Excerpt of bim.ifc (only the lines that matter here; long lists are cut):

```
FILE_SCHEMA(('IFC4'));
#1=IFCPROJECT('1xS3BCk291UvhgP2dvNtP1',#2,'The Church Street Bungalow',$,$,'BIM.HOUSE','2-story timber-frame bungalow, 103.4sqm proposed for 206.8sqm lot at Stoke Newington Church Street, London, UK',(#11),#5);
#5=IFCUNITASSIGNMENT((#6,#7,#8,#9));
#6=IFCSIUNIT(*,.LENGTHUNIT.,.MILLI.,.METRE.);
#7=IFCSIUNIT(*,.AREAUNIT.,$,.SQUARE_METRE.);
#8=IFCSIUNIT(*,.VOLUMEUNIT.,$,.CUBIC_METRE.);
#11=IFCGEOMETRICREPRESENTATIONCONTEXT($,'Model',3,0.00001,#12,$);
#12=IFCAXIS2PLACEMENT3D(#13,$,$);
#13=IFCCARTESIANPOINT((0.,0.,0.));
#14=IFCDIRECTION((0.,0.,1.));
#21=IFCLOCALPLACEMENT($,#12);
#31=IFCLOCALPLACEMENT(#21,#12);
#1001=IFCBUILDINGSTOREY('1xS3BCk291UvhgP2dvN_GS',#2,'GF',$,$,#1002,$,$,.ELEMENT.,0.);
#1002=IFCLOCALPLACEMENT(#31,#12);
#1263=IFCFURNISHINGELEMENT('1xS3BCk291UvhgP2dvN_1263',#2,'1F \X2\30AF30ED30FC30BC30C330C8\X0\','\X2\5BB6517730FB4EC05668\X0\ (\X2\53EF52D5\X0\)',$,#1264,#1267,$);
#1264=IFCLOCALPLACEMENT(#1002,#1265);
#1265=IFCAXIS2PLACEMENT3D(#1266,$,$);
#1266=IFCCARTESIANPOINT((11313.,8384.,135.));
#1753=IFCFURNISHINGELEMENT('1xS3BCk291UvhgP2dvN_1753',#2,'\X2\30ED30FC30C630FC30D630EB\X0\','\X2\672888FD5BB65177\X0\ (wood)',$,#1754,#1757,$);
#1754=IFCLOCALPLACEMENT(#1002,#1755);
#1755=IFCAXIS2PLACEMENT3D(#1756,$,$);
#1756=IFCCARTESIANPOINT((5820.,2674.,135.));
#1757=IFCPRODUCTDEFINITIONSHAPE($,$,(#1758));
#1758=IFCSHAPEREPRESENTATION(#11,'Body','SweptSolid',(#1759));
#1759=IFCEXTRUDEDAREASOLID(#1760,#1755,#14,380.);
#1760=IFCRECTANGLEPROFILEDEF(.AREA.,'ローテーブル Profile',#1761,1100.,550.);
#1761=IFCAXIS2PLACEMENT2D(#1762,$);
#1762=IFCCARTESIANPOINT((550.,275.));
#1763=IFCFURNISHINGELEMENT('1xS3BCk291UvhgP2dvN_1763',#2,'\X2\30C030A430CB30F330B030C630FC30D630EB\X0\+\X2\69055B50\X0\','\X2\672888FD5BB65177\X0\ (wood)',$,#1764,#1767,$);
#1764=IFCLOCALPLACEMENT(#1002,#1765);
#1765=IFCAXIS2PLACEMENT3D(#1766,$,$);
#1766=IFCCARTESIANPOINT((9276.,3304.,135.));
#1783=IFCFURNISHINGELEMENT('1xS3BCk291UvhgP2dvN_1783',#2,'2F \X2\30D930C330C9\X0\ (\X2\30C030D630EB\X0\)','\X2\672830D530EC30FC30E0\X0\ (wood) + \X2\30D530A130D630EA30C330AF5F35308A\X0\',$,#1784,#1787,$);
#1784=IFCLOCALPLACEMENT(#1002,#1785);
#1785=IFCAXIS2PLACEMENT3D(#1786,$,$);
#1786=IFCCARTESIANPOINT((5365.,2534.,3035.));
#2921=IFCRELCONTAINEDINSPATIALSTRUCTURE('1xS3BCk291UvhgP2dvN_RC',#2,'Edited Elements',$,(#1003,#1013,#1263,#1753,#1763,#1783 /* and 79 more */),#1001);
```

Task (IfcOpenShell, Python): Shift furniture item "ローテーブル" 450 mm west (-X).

```python
import ifcopenshell
import ifcopenshell.api.geometry
import ifcopenshell.util.placement

model = ifcopenshell.open("bim.ifc")

item = model.by_guid("1xS3BCk291UvhgP2dvN_1753")
matrix = ifcopenshell.util.placement.get_local_placement(item.ObjectPlacement)
matrix[0, 3] -= 450.0
ifcopenshell.api.geometry.edit_object_placement(model, product=item, matrix=matrix, is_si=False)

print(ifcopenshell.util.placement.get_local_placement(item.ObjectPlacement).round(3) + 0.0)

model.write("bim_v2.ifc")
```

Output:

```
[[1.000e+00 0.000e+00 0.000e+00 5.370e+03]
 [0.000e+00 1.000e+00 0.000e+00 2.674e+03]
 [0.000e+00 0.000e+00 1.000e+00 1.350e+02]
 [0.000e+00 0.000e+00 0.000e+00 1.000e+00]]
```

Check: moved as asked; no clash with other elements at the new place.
